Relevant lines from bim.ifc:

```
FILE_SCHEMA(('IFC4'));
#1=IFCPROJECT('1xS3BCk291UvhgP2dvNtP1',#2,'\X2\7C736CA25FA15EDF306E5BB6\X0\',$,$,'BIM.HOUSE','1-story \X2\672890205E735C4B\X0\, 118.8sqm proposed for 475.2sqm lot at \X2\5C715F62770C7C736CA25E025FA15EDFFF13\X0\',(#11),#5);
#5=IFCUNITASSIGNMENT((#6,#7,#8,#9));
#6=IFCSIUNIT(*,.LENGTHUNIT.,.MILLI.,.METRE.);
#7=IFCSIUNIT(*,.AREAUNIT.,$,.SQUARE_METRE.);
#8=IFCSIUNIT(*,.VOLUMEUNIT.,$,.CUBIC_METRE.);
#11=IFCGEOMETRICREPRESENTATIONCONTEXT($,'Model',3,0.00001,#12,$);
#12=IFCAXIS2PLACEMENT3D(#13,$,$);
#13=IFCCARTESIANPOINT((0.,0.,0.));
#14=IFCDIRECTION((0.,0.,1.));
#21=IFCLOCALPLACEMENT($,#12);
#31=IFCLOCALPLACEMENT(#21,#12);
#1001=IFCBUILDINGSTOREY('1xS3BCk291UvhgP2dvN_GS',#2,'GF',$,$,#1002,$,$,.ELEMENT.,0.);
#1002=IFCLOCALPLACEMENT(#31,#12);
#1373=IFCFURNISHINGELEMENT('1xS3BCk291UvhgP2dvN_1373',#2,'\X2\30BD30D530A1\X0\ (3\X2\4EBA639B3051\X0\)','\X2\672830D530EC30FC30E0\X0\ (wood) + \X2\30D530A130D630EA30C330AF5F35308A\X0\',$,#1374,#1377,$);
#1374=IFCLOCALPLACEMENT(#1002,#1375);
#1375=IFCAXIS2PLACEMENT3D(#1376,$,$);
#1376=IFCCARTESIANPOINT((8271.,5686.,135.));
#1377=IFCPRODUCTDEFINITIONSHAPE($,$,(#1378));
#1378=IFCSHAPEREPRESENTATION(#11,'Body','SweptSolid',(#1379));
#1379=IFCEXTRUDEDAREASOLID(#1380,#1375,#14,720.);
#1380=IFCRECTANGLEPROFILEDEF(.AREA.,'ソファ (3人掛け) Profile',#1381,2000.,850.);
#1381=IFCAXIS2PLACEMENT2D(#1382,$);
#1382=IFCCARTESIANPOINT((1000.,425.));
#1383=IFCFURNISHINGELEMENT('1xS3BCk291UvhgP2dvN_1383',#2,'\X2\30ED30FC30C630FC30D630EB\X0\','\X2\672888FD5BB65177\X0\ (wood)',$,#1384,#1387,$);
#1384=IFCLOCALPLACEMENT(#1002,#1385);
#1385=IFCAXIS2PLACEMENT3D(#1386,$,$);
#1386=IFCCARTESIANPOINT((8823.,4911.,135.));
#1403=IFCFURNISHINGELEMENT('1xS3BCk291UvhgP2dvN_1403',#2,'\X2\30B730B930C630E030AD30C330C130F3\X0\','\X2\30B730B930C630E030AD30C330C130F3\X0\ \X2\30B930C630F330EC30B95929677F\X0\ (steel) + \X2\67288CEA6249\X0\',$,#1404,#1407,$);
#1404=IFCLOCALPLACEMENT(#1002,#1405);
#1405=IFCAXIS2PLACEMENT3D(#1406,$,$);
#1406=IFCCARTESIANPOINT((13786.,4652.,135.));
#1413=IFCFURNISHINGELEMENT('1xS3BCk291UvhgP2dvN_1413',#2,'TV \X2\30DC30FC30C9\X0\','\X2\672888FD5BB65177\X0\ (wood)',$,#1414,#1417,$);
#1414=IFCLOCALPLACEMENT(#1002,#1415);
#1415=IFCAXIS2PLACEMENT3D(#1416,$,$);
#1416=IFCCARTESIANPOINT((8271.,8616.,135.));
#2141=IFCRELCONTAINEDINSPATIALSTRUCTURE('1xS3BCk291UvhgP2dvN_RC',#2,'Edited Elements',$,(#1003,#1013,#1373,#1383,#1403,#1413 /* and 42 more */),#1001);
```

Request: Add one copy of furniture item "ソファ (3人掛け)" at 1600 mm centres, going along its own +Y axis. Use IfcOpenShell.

```python
import ifcopenshell
import ifcopenshell.api.geometry
import ifcopenshell.api.root
import ifcopenshell.util.element
import ifcopenshell.util.placement

model = ifcopenshell.open("bim.ifc")


def reuse_history(source, copy):
    """copy_class also copies each property set's owner history, people and application; keep the originals."""
    for rel in copy.IsDefinedBy:
        if rel.is_a("IfcRelDefinesByProperties") and (history := rel.RelatingPropertyDefinition.OwnerHistory):
            rel.RelatingPropertyDefinition.OwnerHistory = source.OwnerHistory
            ifcopenshell.util.element.remove_deep2(model, history)


source = model.by_guid("1xS3BCk291UvhgP2dvN_1373")
base = ifcopenshell.util.placement.get_local_placement(source.ObjectPlacement)
step = base[:3, 1] * 1600.0

for i in range(1, 2):
    copy = ifcopenshell.api.root.copy_class(model, product=source)
    copy.Representation = ifcopenshell.util.element.copy_deep(
        model, source.Representation, exclude=["IfcGeometricRepresentationContext", "IfcRepresentationMap"]
    )
    reuse_history(source, copy)
    matrix = base.copy()
    matrix[:3, 3] += i * step
    print("added at", matrix[:3, 3].round(3) + 0.0)
    ifcopenshell.api.geometry.edit_object_placement(model, product=copy, matrix=matrix, is_si=False)

model.write("bim_rev.ifc")
```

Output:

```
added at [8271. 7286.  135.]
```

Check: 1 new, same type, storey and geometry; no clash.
